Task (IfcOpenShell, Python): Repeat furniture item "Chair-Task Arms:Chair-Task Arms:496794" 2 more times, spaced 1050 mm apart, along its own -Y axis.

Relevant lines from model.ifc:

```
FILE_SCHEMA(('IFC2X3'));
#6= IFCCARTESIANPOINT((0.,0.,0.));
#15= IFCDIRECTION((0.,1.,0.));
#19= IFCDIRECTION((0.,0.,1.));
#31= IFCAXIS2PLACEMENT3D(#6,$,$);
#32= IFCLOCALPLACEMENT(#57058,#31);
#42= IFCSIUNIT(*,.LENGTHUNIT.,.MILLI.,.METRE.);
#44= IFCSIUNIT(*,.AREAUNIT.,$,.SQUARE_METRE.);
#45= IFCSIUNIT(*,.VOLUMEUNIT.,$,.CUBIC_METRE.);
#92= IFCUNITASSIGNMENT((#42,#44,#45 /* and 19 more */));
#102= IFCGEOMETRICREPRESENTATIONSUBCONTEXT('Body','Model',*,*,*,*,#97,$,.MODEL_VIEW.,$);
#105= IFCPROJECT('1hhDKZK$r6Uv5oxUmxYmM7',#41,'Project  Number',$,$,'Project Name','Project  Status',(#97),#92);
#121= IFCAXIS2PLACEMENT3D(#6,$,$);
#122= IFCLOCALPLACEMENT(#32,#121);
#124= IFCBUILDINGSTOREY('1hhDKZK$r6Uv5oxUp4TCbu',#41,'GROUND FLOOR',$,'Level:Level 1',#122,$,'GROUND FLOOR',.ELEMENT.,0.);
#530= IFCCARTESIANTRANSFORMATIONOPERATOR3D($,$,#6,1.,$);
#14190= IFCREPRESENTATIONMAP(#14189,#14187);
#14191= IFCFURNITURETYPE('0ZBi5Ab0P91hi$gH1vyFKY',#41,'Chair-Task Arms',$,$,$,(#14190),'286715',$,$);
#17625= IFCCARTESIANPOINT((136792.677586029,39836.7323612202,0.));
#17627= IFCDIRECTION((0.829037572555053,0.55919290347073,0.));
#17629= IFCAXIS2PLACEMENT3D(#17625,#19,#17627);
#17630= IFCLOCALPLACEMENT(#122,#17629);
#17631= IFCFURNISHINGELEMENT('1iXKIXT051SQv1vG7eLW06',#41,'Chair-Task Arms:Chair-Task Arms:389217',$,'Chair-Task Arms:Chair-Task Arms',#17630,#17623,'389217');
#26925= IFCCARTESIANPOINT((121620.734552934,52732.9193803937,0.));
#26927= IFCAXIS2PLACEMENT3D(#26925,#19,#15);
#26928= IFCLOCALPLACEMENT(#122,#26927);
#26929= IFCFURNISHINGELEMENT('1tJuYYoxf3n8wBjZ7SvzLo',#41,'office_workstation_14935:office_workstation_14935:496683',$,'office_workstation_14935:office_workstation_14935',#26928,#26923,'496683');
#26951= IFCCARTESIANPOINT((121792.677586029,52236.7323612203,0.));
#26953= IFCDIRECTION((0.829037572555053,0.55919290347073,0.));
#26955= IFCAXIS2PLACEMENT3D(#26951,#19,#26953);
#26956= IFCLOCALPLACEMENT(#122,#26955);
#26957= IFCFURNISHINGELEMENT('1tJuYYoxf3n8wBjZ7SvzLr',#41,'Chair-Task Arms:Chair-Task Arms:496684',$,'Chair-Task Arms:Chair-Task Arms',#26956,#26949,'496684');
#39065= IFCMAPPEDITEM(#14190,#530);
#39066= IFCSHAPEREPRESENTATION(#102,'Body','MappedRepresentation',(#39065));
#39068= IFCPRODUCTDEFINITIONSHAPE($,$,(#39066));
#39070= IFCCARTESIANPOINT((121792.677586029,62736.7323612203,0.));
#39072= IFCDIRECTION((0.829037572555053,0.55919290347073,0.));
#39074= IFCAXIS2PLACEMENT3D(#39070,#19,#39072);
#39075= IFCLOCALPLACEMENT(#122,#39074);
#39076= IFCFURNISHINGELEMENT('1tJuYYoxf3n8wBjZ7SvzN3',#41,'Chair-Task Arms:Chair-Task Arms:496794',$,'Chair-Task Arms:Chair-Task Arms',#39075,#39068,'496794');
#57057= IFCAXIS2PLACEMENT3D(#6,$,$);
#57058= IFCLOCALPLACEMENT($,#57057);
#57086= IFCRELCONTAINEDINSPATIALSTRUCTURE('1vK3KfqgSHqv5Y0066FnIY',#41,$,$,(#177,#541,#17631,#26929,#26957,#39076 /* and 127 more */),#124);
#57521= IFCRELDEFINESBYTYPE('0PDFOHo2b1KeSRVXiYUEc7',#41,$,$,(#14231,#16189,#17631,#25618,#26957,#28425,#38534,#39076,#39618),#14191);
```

```python
import ifcopenshell
import ifcopenshell.api.geometry
import ifcopenshell.api.root
import ifcopenshell.util.element
import ifcopenshell.util.placement
import ifcopenshell.util.unit

model = ifcopenshell.open("model.ifc")
unit_scale = ifcopenshell.util.unit.calculate_unit_scale(model)


def reuse_history(source, copy):
    """copy_class also copies each property set's owner history, people and application; keep the originals."""
    for rel in copy.IsDefinedBy:
        if rel.is_a("IfcRelDefinesByProperties") and (history := rel.RelatingPropertyDefinition.OwnerHistory):
            rel.RelatingPropertyDefinition.OwnerHistory = source.OwnerHistory
            ifcopenshell.util.element.remove_deep2(model, history)


source = model.by_id(39076)
base = ifcopenshell.util.placement.get_local_placement(source.ObjectPlacement)
step = -base[:3, 1] * 1.05 / unit_scale

for i in range(1, 3):
    copy = ifcopenshell.api.root.copy_class(model, product=source)
    copy.Representation = ifcopenshell.util.element.copy_deep(
        model, source.Representation, exclude=["IfcGeometricRepresentationContext", "IfcRepresentationMap"]
    )
    copy.Name = "Chair-Task Arms:Chair-Task Arms"
    copy.Tag = None
    reuse_history(source, copy)
    matrix = base.copy()
    matrix[:3, 3] += i * step
    print("added at", matrix[:3, 3].round(3) + 0.0)
    ifcopenshell.api.geometry.edit_object_placement(model, product=copy, matrix=matrix, is_si=False)

model.write("model_v2.ifc")
```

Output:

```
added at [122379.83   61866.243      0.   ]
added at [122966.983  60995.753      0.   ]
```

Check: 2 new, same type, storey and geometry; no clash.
